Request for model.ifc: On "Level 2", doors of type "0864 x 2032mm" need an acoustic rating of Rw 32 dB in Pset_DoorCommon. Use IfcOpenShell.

First a look at what the model holds.

```python
import ifcopenshell
import ifcopenshell.util.element

model = ifcopenshell.open("model.ifc")
print(model.schema)
storey = next(s for s in model.by_type("IfcBuildingStorey") if s.Name == "Level 2")
doors = [e for e in ifcopenshell.util.element.get_decomposition(storey) if e.is_a("IfcDoor")]
seen = {}
for e in doors:
    element_type = ifcopenshell.util.element.get_type(e)
    key = (element_type.Name if element_type != e and element_type else None, ifcopenshell.util.element.get_pset(e, "Pset_DoorCommon", "AcousticRating"))
    seen[key] = seen.get(key, 0) + 1
for (name, value), count in sorted(seen.items(), key=str):
    print(count, "x", name, "|", value)
```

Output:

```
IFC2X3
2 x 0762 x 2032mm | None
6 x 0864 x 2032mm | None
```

```python
import ifcopenshell
import ifcopenshell.api.pset
import ifcopenshell.util.element

model = ifcopenshell.open("model.ifc")

storey = next(s for s in model.by_type("IfcBuildingStorey") if s.Name == "Level 2")
doors = [e for e in ifcopenshell.util.element.get_decomposition(storey) if e.is_a("IfcDoor")]

count = 0
for e in doors:
    element_type = ifcopenshell.util.element.get_type(e)
    if element_type in (None, e) or element_type.Name != "0864 x 2032mm":
        continue
    # add_pset returns the element's existing set when there is one.
    pset = ifcopenshell.api.pset.add_pset(model, product=e, name="Pset_DoorCommon")
    ifcopenshell.api.pset.edit_pset(model, pset=pset, properties={"AcousticRating": "Rw 32 dB"})
    count += 1

print(count, "doors updated")

model.write("model-out.ifc")
```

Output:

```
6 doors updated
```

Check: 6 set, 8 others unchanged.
